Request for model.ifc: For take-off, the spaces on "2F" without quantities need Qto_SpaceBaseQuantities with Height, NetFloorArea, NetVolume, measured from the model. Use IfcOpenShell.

First a look at what the model holds.

```python
import ifcopenshell
import ifcopenshell.util.element
import ifcopenshell.util.unit

model = ifcopenshell.open("model.ifc")
print(model.schema)
for unit_type in ("LENGTHUNIT", "AREAUNIT", "VOLUMEUNIT"):
    print(unit_type, ifcopenshell.util.unit.calculate_unit_scale(model, unit_type))
storey = next(s for s in model.by_type("IfcBuildingStorey") if s.Name == "2F")
spaces = [e for e in ifcopenshell.util.element.get_decomposition(storey) if e.is_a("IfcSpace")]
for e in sorted(spaces, key=lambda e: e.id()):
    print(e.id(), e.is_a(), e.Name, list(ifcopenshell.util.element.get_psets(e, qtos_only=True)), sep=" | ")
```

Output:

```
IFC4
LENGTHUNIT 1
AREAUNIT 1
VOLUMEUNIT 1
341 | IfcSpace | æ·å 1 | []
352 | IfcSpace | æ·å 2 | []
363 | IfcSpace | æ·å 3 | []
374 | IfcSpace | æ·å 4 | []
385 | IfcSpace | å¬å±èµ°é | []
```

```python
import ifcopenshell
import ifcopenshell.api.pset
import ifcopenshell.geom
import ifcopenshell.util.element
import ifcopenshell.util.shape
import ifcopenshell.util.unit

model = ifcopenshell.open("model.ifc")
unit_scale = ifcopenshell.util.unit.calculate_unit_scale(model)
area_scale = ifcopenshell.util.unit.calculate_unit_scale(model, "AREAUNIT")
volume_scale = ifcopenshell.util.unit.calculate_unit_scale(model, "VOLUMEUNIT")
settings = ifcopenshell.geom.settings()

storey = next(s for s in model.by_type("IfcBuildingStorey") if s.Name == "2F")
spaces = [e for e in ifcopenshell.util.element.get_decomposition(storey) if e.is_a("IfcSpace")]

for e in sorted(spaces, key=lambda e: e.id()):
    if ifcopenshell.util.element.get_psets(e, qtos_only=True, should_inherit=False):
        continue
    # Geometry comes back in metres, in the element's own axes.
    shape = ifcopenshell.geom.create_shape(settings, e)
    values = {
        "Height": ifcopenshell.util.shape.get_z(shape.geometry) / unit_scale,
        "NetFloorArea": ifcopenshell.util.shape.get_footprint_area(shape.geometry) / area_scale,
        "NetVolume": ifcopenshell.util.shape.get_volume(shape.geometry) / volume_scale,
    }
    qto = ifcopenshell.api.pset.add_qto(model, product=e, name="Qto_SpaceBaseQuantities")
    ifcopenshell.api.pset.edit_qto(model, qto=qto, properties=values)
    print(e.id(), {k: round(v, 3) for k, v in values.items()})

model.write("model-out.ifc")
```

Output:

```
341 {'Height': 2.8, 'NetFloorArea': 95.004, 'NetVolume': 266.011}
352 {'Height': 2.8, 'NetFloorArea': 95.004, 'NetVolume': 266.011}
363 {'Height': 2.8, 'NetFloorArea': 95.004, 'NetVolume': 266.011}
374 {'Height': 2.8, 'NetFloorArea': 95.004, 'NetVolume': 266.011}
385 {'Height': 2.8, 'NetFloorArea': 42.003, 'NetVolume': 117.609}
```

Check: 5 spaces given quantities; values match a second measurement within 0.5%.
